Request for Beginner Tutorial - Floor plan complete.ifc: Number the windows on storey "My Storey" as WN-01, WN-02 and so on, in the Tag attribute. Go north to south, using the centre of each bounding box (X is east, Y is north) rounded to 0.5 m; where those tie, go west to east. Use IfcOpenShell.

First a look at what the model holds.

```python
import ifcopenshell
import ifcopenshell.util.element
import ifcopenshell.util.placement

model = ifcopenshell.open("Beginner Tutorial - Floor plan complete.ifc")
print(model.schema)
storey = next(s for s in model.by_type("IfcBuildingStorey") if s.Name == "My Storey")
windows = [e for e in ifcopenshell.util.element.get_decomposition(storey) if e.is_a("IfcWindow")]
for e in sorted(windows, key=lambda e: e.id()):
    origin = ifcopenshell.util.placement.get_local_placement(e.ObjectPlacement)[:3, 3]
    print(e.id(), e.Tag, e.Name, origin.round(2) + 0.0, sep=" | ")
```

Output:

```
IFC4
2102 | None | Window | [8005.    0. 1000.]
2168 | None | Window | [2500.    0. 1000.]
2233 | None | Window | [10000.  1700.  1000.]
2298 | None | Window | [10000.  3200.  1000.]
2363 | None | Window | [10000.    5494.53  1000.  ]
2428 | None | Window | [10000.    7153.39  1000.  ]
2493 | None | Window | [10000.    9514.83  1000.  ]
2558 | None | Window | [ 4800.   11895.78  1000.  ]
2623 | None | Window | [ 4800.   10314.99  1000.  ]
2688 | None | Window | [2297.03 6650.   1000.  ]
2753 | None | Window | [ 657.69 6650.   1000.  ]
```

```python
import ifcopenshell
import ifcopenshell.geom
import ifcopenshell.util.element
import ifcopenshell.util.shape

model = ifcopenshell.open("Beginner Tutorial - Floor plan complete.ifc")
settings = ifcopenshell.geom.settings()
settings.set("use-world-coords", True)


def centre(element):
    shape = ifcopenshell.geom.create_shape(settings, element)
    return ifcopenshell.util.shape.get_bbox_centroid(shape.geometry)


storey = next(s for s in model.by_type("IfcBuildingStorey") if s.Name == "My Storey")
windows = [e for e in ifcopenshell.util.element.get_decomposition(storey) if e.is_a("IfcWindow")]

# Insertion points can sit at a corner or the storey origin, so sort by the geometry (in metres).
centres = {e: centre(e) for e in windows}
windows.sort(key=lambda e: (-round(centres[e][1] / 0.5), centres[e][0]))

for i, e in enumerate(windows, start=1):
    number = f"WN-{i:02d}"
    e.Tag = number
    print(e.id(), number)

model.write("Beginner Tutorial - Floor plan complete_updated.ifc")
```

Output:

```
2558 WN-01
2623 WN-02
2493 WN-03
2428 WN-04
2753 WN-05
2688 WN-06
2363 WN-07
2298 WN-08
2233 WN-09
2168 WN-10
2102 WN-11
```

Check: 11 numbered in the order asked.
